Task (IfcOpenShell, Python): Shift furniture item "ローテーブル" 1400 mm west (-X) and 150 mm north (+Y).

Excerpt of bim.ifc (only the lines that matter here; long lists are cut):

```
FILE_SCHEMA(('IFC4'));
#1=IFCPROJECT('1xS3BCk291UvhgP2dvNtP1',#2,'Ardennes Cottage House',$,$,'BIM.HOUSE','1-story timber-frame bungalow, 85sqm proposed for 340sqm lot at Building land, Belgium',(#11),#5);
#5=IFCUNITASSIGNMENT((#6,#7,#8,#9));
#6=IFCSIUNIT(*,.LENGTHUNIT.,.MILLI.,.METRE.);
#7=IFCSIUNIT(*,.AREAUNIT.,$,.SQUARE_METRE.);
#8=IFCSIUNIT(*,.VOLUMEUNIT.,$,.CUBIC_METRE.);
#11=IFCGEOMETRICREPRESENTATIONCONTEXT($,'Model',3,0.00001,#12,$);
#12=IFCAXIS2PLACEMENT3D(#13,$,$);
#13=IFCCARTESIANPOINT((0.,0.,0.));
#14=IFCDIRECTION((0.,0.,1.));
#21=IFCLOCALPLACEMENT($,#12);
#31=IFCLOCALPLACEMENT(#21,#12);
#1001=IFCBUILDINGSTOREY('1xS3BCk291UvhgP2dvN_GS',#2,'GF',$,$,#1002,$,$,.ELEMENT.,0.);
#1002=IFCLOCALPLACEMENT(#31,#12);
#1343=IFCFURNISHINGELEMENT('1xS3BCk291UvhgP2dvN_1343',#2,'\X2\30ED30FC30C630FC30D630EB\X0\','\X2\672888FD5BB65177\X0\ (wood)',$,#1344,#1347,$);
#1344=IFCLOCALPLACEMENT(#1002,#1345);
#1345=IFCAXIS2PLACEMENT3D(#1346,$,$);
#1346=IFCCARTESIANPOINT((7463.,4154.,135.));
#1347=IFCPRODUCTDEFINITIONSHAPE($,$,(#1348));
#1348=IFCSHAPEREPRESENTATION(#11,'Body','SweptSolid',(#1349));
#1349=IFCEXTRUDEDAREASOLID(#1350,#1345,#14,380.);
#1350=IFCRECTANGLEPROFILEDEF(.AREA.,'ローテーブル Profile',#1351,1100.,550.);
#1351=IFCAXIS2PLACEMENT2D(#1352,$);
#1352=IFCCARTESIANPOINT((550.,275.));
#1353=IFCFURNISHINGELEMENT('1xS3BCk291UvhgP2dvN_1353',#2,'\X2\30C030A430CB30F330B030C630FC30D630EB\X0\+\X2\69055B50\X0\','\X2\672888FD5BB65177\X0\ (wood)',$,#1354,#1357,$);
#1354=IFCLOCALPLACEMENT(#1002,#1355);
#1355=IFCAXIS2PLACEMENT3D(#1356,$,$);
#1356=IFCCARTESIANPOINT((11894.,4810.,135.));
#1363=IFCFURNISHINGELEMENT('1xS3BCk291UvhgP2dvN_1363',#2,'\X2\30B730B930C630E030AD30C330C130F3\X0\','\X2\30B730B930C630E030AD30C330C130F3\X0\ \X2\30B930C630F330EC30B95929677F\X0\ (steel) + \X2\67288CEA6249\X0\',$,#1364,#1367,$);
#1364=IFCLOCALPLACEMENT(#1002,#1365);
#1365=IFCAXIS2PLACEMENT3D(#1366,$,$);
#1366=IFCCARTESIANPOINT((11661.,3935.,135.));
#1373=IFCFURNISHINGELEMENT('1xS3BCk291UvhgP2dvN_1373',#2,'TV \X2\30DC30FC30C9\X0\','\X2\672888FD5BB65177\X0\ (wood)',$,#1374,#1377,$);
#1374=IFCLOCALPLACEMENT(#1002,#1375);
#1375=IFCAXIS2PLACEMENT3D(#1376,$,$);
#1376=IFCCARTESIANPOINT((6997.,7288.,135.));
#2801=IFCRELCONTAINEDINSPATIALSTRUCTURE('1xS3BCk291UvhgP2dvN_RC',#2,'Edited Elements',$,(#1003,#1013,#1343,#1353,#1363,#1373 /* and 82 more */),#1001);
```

```python
import ifcopenshell
import ifcopenshell.api.geometry
import ifcopenshell.util.placement
import ifcopenshell.util.unit

model = ifcopenshell.open("bim.ifc")
unit_scale = ifcopenshell.util.unit.calculate_unit_scale(model)

item = model.by_guid("1xS3BCk291UvhgP2dvN_1343")
matrix = ifcopenshell.util.placement.get_local_placement(item.ObjectPlacement)
matrix[0, 3] -= 1.4 / unit_scale
matrix[1, 3] += 0.15 / unit_scale
ifcopenshell.api.geometry.edit_object_placement(model, product=item, matrix=matrix, is_si=False)

print(ifcopenshell.util.placement.get_local_placement(item.ObjectPlacement).round(3) + 0.0)

model.write("bim-out.ifc")
```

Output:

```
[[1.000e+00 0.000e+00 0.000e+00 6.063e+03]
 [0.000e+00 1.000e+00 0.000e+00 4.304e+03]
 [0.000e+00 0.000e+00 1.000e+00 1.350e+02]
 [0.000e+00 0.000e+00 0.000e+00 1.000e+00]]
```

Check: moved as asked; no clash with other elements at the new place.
